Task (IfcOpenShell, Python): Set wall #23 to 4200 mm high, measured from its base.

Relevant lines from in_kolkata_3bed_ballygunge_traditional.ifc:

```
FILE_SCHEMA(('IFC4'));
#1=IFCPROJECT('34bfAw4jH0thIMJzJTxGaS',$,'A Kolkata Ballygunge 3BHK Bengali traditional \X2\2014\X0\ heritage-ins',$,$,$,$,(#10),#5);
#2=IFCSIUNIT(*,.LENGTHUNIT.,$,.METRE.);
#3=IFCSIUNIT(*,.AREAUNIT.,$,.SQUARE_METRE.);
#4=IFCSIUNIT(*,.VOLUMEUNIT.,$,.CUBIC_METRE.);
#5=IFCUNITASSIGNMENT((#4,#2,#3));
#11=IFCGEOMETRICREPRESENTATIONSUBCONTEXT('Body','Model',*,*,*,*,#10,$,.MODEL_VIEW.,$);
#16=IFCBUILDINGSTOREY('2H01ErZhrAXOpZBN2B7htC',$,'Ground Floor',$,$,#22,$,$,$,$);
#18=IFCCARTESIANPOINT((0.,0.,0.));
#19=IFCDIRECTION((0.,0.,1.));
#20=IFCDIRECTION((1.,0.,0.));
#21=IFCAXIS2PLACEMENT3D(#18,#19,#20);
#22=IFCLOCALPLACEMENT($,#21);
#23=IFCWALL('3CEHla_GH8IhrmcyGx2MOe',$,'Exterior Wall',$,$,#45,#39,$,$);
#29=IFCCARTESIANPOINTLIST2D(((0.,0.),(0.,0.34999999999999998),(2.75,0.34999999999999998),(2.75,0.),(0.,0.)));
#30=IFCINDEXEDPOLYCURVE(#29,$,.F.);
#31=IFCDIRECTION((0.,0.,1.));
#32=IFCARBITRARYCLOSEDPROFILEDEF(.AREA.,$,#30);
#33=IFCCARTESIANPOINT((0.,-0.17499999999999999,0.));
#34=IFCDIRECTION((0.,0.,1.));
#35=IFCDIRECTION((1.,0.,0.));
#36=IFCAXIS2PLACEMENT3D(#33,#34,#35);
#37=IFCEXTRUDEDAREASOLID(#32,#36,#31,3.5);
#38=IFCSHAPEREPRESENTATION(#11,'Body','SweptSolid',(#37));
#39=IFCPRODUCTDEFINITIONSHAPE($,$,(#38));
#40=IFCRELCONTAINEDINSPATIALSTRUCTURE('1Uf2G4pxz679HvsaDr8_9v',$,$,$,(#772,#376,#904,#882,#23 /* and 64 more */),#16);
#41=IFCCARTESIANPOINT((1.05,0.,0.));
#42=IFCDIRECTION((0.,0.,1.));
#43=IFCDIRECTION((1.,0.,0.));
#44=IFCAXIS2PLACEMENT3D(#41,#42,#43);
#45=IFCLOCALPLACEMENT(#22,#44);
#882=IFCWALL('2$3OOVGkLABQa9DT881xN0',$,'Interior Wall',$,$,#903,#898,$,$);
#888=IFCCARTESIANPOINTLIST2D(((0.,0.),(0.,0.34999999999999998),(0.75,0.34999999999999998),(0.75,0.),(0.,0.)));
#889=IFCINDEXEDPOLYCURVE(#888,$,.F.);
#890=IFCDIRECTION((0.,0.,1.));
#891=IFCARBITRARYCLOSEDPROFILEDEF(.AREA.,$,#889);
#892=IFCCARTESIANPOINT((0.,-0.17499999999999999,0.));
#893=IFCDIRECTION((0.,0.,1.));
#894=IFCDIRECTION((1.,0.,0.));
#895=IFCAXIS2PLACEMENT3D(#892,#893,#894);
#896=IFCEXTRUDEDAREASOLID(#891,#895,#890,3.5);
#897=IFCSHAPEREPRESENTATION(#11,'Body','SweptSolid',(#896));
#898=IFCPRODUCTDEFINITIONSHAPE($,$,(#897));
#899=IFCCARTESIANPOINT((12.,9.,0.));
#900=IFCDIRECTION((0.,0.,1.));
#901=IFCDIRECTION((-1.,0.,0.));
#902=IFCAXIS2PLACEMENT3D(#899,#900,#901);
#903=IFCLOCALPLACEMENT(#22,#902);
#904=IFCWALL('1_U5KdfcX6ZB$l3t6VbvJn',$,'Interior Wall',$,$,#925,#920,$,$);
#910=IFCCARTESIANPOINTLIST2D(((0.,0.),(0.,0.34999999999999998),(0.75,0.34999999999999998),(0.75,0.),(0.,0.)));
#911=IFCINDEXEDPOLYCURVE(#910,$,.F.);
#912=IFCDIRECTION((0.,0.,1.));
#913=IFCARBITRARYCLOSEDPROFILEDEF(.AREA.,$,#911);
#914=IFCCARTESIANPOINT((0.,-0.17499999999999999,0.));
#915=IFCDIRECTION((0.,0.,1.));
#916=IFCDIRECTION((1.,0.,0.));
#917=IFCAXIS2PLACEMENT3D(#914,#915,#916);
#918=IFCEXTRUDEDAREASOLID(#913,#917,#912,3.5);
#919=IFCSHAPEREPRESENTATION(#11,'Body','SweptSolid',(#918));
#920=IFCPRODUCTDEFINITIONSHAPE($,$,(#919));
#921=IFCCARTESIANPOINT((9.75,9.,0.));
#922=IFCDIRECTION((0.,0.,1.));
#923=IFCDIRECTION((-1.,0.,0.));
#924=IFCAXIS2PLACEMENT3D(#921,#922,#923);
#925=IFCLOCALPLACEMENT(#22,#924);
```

```python
import ifcopenshell
import ifcopenshell.geom
import ifcopenshell.util.representation
import ifcopenshell.util.shape

model = ifcopenshell.open("in_kolkata_3bed_ballygunge_traditional.ifc")
settings = ifcopenshell.geom.settings()


def volume(element):
    """Net volume in cubic metres, openings subtracted."""
    shape = ifcopenshell.geom.create_shape(settings, element)
    return ifcopenshell.util.shape.get_volume(shape.geometry)


wall = model.by_guid("3CEHla_GH8IhrmcyGx2MOe")
before = volume(wall)

body = ifcopenshell.util.representation.get_representation(wall, "Model", "Body")
solid = body.Items[0]
old_height = solid.Depth
solid.Depth = 4.2
after = volume(wall)

print(f"height {old_height:g} -> {solid.Depth:g}, volume {before:.3f} -> {after:.3f} m3")

model.write("in_kolkata_3bed_ballygunge_traditional_edited.ifc")
```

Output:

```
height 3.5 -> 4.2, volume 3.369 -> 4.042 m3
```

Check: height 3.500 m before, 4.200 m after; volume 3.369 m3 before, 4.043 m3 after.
